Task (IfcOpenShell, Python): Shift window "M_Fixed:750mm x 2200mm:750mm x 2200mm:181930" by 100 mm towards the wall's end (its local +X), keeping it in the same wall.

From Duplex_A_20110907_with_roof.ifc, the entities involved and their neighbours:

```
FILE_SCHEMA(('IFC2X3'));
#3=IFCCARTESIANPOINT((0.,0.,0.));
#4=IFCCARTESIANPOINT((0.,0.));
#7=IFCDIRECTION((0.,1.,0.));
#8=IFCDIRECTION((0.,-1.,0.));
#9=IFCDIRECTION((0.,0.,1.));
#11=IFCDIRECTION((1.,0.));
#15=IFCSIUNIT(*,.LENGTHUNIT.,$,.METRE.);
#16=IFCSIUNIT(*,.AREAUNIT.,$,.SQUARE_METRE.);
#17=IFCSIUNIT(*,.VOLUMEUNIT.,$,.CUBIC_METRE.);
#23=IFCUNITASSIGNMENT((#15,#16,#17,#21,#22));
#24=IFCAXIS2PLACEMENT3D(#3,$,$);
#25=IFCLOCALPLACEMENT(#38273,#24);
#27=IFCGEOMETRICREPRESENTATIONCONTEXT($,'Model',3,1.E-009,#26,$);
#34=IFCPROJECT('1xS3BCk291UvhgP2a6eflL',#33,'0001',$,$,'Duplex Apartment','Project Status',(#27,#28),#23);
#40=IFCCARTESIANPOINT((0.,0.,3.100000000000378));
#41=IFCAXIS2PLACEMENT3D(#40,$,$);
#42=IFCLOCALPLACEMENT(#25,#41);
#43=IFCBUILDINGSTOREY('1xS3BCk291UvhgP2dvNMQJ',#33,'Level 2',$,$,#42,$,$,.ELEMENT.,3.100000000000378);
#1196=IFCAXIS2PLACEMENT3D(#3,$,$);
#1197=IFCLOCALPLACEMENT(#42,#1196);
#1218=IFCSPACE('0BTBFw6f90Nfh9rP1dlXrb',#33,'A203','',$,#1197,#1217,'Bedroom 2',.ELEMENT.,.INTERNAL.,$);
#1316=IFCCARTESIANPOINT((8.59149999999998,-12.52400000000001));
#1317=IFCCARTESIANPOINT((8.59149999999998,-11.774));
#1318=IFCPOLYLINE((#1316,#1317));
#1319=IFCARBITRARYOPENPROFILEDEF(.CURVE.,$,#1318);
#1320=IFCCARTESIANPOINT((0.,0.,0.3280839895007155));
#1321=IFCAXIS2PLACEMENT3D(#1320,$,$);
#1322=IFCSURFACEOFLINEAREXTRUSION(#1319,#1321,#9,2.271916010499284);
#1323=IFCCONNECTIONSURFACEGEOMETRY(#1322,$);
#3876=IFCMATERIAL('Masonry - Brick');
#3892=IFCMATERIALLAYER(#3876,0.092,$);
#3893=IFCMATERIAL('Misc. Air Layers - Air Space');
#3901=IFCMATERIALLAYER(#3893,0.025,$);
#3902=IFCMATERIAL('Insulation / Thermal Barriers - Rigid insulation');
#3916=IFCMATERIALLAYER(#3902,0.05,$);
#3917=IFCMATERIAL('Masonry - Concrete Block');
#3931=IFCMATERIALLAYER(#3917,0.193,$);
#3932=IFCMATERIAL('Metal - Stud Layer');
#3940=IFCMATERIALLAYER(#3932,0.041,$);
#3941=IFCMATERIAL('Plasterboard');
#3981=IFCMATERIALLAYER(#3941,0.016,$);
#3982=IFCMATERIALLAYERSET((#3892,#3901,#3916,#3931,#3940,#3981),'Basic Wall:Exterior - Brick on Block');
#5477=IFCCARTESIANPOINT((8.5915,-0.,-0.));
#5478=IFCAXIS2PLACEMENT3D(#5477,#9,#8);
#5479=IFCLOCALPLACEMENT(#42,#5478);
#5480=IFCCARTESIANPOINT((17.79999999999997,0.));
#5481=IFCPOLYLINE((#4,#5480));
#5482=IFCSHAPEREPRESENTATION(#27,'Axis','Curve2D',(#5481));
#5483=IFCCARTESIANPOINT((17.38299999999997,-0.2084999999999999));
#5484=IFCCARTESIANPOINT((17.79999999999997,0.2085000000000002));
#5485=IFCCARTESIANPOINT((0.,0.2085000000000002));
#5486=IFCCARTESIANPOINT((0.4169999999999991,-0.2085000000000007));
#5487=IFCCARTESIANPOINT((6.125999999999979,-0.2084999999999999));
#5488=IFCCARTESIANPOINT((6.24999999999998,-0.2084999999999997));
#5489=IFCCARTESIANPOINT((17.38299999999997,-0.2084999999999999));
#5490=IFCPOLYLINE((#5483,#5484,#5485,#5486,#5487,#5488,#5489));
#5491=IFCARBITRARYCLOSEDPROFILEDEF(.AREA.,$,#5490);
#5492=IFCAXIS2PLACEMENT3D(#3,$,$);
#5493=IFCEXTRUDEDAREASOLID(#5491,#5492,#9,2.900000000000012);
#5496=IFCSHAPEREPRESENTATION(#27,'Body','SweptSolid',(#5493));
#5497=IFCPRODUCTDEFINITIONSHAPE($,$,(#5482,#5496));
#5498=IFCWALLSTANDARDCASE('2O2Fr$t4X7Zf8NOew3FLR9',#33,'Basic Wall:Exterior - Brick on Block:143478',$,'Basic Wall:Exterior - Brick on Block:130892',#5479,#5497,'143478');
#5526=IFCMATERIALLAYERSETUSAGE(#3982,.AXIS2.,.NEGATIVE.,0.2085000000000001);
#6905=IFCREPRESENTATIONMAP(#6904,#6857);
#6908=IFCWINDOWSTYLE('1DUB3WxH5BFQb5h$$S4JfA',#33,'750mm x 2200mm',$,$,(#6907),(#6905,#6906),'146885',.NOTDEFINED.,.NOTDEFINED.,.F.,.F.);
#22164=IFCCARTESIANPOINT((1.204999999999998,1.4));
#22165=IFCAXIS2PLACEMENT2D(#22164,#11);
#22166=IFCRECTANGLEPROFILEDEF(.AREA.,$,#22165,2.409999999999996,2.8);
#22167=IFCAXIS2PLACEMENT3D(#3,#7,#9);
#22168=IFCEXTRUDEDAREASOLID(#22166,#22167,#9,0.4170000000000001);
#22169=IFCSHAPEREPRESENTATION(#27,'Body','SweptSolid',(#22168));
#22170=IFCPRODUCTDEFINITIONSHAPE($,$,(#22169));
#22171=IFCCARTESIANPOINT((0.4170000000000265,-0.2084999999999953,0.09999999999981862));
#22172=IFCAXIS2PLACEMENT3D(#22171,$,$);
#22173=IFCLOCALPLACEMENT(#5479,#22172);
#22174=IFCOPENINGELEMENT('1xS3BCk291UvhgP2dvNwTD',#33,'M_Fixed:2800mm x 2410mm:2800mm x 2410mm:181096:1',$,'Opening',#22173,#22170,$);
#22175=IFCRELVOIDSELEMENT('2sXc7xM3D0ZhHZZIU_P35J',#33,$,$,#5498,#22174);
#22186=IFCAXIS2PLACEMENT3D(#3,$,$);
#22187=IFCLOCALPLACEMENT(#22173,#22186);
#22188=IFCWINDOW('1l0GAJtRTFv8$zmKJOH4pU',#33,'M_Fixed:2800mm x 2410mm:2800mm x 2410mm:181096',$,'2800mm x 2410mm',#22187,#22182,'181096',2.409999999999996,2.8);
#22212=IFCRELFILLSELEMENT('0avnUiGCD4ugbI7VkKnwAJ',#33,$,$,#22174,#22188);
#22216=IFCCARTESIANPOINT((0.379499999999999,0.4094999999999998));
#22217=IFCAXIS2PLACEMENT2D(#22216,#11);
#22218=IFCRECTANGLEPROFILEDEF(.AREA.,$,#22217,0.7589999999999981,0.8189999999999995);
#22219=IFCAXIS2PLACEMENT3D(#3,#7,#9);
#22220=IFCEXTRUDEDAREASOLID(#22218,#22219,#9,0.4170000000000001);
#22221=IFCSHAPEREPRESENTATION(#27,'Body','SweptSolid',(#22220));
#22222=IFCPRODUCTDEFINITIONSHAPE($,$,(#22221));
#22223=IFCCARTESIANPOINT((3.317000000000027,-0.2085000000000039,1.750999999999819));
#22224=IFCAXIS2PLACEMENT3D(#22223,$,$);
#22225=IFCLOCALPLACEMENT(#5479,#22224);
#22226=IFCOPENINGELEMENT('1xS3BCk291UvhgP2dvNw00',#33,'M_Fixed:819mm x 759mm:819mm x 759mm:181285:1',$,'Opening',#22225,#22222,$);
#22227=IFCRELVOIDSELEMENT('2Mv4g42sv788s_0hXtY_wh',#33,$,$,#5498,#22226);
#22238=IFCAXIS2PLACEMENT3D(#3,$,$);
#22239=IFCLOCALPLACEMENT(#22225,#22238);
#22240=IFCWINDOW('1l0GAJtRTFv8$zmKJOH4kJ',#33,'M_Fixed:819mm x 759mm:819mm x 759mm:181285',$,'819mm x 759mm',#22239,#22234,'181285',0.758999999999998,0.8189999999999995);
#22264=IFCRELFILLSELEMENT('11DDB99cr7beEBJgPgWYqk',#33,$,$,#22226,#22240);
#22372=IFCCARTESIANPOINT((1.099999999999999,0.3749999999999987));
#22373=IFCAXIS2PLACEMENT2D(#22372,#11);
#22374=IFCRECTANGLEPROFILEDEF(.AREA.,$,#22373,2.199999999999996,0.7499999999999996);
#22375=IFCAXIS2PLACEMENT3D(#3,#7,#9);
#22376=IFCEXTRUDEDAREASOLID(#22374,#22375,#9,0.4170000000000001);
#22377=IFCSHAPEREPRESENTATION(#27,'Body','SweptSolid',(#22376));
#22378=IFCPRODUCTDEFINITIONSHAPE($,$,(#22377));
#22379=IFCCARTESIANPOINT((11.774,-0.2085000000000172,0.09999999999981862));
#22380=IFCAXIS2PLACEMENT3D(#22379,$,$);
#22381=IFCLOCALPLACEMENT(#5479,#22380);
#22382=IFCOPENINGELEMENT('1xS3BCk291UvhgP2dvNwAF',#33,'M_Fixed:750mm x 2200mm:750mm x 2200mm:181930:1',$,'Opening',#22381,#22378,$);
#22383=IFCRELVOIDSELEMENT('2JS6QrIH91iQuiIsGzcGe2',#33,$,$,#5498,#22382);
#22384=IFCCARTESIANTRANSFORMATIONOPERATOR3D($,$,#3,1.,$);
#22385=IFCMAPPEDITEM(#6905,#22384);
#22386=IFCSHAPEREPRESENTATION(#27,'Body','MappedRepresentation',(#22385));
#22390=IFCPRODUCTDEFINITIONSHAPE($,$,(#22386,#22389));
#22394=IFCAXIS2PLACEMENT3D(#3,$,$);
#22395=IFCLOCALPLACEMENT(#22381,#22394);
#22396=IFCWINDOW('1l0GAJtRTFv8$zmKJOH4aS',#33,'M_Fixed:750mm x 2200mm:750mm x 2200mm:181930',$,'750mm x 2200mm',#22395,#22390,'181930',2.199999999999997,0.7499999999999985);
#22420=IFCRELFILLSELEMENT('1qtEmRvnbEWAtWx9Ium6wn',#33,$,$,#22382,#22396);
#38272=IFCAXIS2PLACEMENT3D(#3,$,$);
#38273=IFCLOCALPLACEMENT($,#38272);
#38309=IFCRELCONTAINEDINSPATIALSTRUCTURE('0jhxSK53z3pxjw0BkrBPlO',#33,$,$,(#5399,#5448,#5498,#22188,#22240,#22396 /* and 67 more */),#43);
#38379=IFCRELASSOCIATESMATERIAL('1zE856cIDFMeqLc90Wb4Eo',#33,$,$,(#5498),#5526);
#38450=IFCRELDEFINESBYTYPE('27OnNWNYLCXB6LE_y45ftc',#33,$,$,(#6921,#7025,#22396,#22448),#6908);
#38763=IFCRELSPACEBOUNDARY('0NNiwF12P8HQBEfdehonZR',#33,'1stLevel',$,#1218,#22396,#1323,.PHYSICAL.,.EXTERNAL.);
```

```python
import numpy as np
import ifcopenshell
import ifcopenshell.api.geometry
import ifcopenshell.util.placement

model = ifcopenshell.open("Duplex_A_20110907_with_roof.ifc")

window = model.by_id(22396)
opening = window.FillsVoids[0].RelatingOpeningElement
wall = opening.VoidsElements[0].RelatingBuildingElement

wall_matrix = ifcopenshell.util.placement.get_local_placement(wall.ObjectPlacement)
shift = wall_matrix[:3, 0] * 0.1
before = ifcopenshell.util.placement.get_local_placement(window.ObjectPlacement)[:3, 3].copy()

# The window is placed relative to its opening, so it follows when the opening moves.
matrix = ifcopenshell.util.placement.get_local_placement(opening.ObjectPlacement)
matrix[:3, 3] += shift
ifcopenshell.api.geometry.edit_object_placement(
    model, product=opening, matrix=matrix, is_si=False, should_transform_children=True
)

# Space boundary surfaces are stored in each space's coordinates; move them too.
for rel in window.ProvidesBoundaries:
    if not rel.ConnectionGeometry:
        continue
    surface = rel.ConnectionGeometry.SurfaceOnRelatingElement
    space_matrix = ifcopenshell.util.placement.get_local_placement(rel.RelatingSpace.ObjectPlacement)
    point = np.array(surface.Position.Location.Coordinates) + space_matrix[:3, :3].T @ shift
    surface.Position = model.createIfcAxis2Placement3D(
        model.createIfcCartesianPoint(point.tolist()), surface.Position.Axis, surface.Position.RefDirection
    )

after = ifcopenshell.util.placement.get_local_placement(window.ObjectPlacement)[:3, 3]
print("window moved by", (after - before).round(3) + 0.0)

model.write("Duplex_A_20110907_with_roof_v2.ifc")
```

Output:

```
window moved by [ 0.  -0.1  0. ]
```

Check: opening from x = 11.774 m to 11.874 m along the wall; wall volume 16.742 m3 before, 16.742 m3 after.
